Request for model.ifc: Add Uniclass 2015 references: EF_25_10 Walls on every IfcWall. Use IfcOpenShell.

First a look at what the model holds.

```python
import ifcopenshell

model = ifcopenshell.open("model.ifc")
print(model.schema)
print("classifications:", [c.Name for c in model.by_type("IfcClassification")])
for ifc_class in ("IfcDoor", "IfcRoof", "IfcStair", "IfcWall", "IfcWindow"):
    print(ifc_class, len(model.by_type(ifc_class)))
```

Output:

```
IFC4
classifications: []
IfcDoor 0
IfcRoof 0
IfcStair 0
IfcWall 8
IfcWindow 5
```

```python
import ifcopenshell
import ifcopenshell.api.classification

model = ifcopenshell.open("model.ifc")

system = ifcopenshell.api.classification.add_classification(model, classification="Uniclass 2015")

codes = {
    "IfcWall": ("EF_25_10", "Walls"),
}
for ifc_class, (code, name) in codes.items():
    products = model.by_type(ifc_class)
    ifcopenshell.api.classification.add_reference(
        model, products=products, classification=system, identification=code, name=name
    )
    print(code, len(products))

model.write("model-out.ifc")
```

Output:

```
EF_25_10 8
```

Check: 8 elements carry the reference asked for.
